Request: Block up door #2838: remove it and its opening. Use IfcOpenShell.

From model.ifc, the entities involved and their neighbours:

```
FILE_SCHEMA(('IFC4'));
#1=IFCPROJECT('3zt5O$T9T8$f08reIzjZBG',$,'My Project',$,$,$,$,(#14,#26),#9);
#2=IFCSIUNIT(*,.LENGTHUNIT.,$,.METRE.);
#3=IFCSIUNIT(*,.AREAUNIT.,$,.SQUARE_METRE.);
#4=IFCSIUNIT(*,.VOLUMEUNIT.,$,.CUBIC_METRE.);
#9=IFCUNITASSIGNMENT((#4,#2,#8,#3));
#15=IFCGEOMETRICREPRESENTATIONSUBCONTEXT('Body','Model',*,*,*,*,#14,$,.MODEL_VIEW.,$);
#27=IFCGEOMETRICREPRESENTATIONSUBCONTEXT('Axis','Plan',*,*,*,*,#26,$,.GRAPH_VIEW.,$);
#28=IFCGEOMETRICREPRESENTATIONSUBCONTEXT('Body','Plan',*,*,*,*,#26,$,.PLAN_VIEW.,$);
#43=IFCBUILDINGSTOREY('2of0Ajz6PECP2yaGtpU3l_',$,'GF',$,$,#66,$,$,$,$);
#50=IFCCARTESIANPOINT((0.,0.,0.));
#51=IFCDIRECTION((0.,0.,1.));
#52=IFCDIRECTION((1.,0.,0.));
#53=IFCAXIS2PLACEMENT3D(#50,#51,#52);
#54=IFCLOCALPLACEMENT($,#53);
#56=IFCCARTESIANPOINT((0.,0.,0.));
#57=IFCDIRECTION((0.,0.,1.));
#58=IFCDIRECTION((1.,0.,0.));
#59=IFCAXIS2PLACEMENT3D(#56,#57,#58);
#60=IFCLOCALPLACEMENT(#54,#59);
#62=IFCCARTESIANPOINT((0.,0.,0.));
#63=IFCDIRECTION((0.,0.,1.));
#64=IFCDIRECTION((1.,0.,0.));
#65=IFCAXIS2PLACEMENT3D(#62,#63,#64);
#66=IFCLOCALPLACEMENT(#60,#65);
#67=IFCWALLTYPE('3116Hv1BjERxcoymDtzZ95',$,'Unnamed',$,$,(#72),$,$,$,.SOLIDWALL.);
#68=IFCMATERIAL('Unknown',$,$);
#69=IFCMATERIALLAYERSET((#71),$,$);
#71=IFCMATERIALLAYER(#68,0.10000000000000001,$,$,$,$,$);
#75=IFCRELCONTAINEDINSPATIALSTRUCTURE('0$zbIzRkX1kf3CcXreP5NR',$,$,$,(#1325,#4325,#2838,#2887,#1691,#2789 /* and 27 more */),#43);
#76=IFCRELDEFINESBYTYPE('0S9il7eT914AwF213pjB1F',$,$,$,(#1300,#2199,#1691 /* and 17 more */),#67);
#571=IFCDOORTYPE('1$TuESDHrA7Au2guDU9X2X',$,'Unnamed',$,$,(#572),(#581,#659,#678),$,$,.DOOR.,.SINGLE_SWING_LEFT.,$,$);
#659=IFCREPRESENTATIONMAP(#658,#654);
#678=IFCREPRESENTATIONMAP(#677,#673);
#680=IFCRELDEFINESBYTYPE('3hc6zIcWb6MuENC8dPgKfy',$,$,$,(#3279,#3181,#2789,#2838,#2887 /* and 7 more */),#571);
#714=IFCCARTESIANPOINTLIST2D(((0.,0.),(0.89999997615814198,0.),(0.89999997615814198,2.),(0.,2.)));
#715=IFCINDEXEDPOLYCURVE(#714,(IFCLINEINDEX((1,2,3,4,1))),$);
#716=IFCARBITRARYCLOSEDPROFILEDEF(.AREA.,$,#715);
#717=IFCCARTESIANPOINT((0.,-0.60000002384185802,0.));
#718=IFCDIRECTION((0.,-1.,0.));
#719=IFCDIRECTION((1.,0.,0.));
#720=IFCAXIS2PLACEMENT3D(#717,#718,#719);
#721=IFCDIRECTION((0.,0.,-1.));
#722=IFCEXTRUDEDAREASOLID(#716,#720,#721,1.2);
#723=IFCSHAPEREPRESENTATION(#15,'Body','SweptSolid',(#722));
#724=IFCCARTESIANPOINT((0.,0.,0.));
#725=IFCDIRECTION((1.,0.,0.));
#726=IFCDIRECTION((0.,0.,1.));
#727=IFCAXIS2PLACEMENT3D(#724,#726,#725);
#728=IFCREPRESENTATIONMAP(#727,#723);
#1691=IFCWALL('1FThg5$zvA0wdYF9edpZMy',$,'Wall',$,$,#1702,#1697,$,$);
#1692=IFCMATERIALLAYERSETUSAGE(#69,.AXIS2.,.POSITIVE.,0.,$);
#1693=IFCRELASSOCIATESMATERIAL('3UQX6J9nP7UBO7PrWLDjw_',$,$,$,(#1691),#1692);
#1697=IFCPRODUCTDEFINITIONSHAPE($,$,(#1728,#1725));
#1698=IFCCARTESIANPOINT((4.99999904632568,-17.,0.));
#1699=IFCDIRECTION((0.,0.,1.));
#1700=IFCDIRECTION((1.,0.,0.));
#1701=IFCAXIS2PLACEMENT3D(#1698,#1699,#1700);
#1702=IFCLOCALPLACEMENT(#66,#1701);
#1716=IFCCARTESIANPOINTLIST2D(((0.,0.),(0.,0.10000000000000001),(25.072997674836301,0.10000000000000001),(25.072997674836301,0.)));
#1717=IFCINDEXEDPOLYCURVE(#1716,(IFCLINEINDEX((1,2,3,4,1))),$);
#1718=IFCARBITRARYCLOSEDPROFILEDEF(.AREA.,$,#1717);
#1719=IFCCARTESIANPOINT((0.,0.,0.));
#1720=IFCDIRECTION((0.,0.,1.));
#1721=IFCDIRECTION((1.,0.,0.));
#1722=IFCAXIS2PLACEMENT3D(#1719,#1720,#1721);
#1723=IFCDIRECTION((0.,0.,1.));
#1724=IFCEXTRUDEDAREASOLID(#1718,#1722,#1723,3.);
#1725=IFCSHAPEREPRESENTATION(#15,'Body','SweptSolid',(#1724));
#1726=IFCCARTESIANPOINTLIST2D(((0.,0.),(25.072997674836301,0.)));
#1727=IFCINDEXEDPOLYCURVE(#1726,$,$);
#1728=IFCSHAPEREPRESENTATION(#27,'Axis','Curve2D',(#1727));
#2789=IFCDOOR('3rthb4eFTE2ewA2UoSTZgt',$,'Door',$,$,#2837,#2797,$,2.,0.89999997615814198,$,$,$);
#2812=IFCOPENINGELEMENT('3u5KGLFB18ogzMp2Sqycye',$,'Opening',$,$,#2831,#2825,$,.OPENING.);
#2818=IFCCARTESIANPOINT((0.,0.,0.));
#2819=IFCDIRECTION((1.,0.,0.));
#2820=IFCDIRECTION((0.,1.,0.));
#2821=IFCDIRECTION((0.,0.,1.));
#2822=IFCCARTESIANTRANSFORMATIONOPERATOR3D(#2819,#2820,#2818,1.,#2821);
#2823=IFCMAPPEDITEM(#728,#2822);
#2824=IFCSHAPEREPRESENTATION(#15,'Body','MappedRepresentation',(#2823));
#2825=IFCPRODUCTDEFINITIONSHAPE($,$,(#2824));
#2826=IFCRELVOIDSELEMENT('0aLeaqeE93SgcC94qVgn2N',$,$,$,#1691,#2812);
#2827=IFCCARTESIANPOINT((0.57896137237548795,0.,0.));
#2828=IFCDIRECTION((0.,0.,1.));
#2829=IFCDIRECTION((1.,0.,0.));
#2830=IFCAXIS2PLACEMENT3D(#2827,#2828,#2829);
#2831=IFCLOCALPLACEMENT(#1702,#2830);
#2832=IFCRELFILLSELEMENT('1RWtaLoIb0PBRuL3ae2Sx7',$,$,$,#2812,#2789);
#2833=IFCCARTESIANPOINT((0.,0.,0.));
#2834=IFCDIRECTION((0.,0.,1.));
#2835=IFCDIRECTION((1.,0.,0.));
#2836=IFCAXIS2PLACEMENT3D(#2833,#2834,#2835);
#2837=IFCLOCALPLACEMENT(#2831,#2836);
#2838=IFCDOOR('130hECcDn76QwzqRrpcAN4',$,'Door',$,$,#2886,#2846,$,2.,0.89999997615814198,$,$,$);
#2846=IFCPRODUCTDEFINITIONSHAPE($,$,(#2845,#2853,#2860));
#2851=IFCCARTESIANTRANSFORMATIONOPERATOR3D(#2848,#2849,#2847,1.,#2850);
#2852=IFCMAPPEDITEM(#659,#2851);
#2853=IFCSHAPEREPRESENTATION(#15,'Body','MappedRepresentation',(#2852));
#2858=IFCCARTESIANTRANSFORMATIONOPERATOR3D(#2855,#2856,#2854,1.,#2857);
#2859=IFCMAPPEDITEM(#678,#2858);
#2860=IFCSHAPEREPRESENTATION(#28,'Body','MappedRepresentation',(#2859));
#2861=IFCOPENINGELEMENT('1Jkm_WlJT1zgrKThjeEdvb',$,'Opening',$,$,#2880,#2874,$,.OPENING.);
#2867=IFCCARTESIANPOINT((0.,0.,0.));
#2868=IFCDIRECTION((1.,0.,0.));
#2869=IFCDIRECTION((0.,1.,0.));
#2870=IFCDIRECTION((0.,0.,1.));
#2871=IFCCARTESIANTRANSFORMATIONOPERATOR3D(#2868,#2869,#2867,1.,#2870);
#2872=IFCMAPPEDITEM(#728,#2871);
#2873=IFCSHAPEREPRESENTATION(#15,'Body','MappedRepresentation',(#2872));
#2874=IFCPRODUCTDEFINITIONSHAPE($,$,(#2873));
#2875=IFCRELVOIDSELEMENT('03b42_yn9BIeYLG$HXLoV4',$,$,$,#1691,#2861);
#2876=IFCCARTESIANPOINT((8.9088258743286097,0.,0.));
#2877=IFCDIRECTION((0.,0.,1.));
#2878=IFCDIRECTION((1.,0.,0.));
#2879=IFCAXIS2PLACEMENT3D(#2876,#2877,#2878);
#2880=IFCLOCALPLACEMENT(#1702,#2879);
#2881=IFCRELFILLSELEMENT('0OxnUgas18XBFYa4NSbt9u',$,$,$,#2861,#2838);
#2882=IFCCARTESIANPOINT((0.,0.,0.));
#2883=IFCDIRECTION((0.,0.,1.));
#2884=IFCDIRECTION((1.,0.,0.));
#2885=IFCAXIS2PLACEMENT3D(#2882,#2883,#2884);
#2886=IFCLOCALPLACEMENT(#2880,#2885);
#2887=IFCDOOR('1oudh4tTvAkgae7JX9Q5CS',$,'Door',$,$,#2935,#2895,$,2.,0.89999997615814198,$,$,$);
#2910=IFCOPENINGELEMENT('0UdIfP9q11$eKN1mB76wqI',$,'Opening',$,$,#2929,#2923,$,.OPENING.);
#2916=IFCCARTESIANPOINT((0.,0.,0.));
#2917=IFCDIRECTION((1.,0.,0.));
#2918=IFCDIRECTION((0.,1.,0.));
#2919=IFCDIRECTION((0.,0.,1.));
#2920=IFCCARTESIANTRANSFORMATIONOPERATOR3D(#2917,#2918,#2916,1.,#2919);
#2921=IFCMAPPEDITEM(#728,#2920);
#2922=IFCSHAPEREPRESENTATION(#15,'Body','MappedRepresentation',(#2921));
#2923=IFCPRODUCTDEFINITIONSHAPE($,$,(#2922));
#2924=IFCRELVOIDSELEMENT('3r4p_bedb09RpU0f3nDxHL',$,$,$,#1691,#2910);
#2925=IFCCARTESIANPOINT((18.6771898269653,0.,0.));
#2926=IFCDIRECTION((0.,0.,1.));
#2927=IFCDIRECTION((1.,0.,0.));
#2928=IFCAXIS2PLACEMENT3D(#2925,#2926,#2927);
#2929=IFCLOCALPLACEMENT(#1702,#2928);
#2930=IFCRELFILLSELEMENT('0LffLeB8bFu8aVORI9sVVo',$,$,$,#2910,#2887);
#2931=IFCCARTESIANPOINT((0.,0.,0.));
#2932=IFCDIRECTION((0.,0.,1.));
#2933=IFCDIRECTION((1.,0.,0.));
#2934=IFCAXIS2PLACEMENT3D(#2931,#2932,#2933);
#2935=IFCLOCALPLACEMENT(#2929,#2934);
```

```python
import ifcopenshell
import ifcopenshell.api.feature
import ifcopenshell.api.root
import ifcopenshell.geom
import ifcopenshell.util.shape

model = ifcopenshell.open("model.ifc")
settings = ifcopenshell.geom.settings()


def volume(element):
    """Net volume in cubic metres, openings subtracted."""
    shape = ifcopenshell.geom.create_shape(settings, element)
    return ifcopenshell.util.shape.get_volume(shape.geometry)


door = model.by_guid("130hECcDn76QwzqRrpcAN4")
opening = door.FillsVoids[0].RelatingOpeningElement
wall = opening.VoidsElements[0].RelatingBuildingElement
before = volume(wall)

ifcopenshell.api.root.remove_product(model, product=door)
ifcopenshell.api.feature.remove_feature(model, feature=opening)

after = volume(wall)

print(f"wall volume {before:.3f} -> {after:.3f} m3")

model.write("model_v2.ifc")
```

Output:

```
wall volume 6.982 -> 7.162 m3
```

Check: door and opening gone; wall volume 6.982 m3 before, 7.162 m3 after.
